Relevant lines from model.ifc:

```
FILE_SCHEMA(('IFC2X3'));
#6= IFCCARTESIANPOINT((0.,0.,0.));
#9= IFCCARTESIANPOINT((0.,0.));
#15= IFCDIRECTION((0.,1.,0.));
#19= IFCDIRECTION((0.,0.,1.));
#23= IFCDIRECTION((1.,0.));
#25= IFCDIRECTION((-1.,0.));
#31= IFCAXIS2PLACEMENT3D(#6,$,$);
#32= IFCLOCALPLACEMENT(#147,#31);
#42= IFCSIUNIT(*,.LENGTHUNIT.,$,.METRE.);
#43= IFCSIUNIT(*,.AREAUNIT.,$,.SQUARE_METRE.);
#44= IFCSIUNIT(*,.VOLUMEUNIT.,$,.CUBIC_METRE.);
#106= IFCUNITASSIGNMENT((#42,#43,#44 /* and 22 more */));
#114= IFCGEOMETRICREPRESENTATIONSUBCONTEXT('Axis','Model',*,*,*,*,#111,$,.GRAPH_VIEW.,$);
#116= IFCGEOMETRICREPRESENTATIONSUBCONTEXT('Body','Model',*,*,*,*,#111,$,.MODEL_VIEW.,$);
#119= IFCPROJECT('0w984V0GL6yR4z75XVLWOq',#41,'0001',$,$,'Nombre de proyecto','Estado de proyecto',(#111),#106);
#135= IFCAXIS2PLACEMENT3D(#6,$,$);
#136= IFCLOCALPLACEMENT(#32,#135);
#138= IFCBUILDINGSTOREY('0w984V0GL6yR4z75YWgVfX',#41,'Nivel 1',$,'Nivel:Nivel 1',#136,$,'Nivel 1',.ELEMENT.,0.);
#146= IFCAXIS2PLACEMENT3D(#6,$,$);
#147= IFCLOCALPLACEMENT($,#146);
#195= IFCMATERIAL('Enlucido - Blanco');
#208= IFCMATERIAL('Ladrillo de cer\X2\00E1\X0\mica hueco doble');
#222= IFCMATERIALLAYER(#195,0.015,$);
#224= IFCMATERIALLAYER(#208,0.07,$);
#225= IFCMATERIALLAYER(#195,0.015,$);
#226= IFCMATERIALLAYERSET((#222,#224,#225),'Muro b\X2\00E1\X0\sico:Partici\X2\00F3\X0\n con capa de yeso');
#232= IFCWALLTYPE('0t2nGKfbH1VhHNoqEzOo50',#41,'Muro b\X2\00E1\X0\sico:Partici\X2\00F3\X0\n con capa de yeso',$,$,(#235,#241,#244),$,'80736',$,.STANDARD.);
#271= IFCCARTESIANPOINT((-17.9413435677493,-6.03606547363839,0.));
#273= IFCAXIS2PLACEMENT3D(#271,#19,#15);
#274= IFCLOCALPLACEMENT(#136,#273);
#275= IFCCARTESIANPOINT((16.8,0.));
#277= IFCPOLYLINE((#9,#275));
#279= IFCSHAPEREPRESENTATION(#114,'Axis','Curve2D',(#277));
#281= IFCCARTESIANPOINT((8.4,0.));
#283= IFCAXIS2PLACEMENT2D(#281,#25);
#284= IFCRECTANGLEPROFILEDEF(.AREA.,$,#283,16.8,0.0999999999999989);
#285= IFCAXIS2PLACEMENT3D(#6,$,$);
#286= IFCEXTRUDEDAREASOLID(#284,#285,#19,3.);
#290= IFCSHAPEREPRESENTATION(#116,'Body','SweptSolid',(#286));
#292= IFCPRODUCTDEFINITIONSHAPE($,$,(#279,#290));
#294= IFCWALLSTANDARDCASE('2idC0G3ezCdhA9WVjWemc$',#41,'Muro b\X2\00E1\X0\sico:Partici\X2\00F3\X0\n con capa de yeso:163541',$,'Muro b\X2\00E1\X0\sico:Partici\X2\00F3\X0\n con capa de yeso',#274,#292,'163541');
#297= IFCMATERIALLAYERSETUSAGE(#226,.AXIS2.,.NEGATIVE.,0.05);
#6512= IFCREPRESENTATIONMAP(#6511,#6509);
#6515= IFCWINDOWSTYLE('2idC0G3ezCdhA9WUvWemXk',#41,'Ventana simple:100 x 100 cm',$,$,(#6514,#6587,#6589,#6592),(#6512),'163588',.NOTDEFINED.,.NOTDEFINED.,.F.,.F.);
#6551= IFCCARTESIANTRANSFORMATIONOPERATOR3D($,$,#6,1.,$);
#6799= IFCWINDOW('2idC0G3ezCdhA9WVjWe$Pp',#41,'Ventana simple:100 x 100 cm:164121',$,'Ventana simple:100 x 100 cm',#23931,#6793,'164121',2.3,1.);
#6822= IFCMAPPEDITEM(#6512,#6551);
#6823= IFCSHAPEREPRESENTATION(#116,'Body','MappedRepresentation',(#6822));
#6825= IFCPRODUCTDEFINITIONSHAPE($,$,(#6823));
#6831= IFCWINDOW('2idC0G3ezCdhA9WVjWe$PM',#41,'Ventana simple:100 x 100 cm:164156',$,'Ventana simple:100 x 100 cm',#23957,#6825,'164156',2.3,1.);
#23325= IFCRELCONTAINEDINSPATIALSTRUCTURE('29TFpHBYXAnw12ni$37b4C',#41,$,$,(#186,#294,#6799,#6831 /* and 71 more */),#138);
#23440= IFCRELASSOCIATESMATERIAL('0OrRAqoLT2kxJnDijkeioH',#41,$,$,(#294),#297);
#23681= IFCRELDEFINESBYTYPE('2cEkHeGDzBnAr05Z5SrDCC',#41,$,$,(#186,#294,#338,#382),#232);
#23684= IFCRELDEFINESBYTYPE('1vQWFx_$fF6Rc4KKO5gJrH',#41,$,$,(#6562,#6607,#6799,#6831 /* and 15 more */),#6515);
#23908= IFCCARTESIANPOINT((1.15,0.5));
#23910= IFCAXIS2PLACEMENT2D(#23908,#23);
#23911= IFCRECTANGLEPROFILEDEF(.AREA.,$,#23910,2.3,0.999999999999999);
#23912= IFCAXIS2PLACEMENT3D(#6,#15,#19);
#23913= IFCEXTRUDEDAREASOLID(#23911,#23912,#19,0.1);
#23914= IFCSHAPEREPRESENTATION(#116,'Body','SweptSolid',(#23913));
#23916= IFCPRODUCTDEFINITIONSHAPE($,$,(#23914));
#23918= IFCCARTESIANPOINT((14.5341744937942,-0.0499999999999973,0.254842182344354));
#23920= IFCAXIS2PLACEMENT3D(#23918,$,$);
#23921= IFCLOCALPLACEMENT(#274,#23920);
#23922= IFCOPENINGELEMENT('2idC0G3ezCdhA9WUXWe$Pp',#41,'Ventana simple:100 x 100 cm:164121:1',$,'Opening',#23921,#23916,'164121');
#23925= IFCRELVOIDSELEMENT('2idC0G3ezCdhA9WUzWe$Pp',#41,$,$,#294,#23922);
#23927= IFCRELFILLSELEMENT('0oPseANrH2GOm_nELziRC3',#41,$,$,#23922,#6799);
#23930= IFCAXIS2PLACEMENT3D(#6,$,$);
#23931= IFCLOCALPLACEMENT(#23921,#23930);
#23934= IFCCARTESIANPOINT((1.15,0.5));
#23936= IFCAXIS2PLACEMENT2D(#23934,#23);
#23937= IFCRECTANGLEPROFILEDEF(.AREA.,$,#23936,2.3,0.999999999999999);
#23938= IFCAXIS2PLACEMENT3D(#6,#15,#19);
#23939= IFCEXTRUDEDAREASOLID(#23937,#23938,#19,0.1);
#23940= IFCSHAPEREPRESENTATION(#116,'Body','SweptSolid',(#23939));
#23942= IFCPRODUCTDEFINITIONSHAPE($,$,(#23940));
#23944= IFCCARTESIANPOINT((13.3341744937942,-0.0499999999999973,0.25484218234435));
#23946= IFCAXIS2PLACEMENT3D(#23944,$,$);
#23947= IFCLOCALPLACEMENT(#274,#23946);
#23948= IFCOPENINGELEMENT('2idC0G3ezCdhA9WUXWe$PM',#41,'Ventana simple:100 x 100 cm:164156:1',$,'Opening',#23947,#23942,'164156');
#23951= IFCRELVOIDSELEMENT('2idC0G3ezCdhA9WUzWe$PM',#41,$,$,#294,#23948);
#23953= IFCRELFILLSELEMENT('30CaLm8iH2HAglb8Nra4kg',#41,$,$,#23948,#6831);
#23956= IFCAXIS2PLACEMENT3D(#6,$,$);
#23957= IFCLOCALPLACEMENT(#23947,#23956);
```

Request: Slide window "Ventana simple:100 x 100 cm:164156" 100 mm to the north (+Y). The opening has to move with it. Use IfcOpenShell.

```python
import ifcopenshell
import ifcopenshell.api.geometry
import ifcopenshell.util.placement

model = ifcopenshell.open("model.ifc")

window = model.by_guid("2idC0G3ezCdhA9WVjWe$PM")
opening = window.FillsVoids[0].RelatingOpeningElement
wall = opening.VoidsElements[0].RelatingBuildingElement

wall_matrix = ifcopenshell.util.placement.get_local_placement(wall.ObjectPlacement)
shift = wall_matrix[:3, 0] * 0.1
before = ifcopenshell.util.placement.get_local_placement(window.ObjectPlacement)[:3, 3].copy()

# The window is placed relative to its opening, so it follows when the opening moves.
matrix = ifcopenshell.util.placement.get_local_placement(opening.ObjectPlacement)
matrix[:3, 3] += shift
ifcopenshell.api.geometry.edit_object_placement(
    model, product=opening, matrix=matrix, is_si=False, should_transform_children=True
)

after = ifcopenshell.util.placement.get_local_placement(window.ObjectPlacement)[:3, 3]
print("window moved by", (after - before).round(3) + 0.0)

model.write("model_updated.ifc")
```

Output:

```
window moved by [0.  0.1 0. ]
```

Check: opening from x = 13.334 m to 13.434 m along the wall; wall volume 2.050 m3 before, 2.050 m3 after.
